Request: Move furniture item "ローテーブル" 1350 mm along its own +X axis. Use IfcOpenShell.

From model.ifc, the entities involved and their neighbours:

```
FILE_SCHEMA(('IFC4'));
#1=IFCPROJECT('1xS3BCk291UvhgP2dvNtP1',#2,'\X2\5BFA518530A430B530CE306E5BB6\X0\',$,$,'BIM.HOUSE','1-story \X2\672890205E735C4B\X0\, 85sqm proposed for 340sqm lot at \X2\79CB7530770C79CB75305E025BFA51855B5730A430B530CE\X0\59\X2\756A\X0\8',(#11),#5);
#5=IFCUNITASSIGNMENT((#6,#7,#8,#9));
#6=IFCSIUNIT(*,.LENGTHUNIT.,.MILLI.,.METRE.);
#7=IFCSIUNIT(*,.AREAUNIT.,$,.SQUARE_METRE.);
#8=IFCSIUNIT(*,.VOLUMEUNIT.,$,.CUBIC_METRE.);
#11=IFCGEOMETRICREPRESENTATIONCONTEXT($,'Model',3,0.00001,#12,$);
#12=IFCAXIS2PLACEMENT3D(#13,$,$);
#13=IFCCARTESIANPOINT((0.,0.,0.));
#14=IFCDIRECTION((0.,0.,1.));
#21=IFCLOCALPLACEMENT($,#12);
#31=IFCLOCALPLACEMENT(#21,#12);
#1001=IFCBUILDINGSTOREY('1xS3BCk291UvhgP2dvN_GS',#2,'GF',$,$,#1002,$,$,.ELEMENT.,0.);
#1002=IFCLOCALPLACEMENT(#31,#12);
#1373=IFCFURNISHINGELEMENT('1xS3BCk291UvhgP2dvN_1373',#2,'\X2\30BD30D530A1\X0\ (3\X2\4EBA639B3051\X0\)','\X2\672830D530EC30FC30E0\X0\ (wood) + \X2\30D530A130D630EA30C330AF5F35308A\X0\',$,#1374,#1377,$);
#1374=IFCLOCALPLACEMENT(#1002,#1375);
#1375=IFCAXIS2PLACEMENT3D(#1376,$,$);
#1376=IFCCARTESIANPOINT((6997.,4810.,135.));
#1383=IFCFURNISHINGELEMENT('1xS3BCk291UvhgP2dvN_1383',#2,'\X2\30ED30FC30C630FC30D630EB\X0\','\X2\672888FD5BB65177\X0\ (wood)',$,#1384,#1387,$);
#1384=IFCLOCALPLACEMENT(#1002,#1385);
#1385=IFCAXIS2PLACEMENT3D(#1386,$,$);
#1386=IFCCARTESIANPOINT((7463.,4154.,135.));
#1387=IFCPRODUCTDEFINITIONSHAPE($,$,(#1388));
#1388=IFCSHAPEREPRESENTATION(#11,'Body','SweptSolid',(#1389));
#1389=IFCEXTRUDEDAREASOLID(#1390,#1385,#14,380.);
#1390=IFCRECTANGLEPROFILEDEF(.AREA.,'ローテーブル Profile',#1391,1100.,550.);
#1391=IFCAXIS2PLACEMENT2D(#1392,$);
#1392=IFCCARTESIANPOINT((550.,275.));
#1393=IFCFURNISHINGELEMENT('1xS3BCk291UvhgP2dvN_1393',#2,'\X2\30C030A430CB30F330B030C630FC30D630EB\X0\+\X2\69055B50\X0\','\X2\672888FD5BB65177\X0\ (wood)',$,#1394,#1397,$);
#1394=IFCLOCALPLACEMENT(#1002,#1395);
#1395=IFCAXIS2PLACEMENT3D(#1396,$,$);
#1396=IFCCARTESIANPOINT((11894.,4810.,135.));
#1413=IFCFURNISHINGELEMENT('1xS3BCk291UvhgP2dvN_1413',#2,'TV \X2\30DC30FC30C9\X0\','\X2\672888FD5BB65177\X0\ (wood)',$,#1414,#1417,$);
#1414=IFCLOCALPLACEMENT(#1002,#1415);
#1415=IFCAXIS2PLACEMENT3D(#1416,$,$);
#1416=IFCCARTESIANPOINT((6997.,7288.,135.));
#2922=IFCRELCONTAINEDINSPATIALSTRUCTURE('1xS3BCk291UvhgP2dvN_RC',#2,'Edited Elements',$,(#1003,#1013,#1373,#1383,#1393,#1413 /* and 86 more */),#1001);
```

```python
import ifcopenshell
import ifcopenshell.api.geometry
import ifcopenshell.util.placement
import ifcopenshell.util.unit

model = ifcopenshell.open("model.ifc")
unit_scale = ifcopenshell.util.unit.calculate_unit_scale(model)

item = model.by_guid("1xS3BCk291UvhgP2dvN_1383")
matrix = ifcopenshell.util.placement.get_local_placement(item.ObjectPlacement)
matrix[:3, 3] += matrix[:3, 0] * 1.35 / unit_scale
ifcopenshell.api.geometry.edit_object_placement(model, product=item, matrix=matrix, is_si=False)

print(ifcopenshell.util.placement.get_local_placement(item.ObjectPlacement).round(3) + 0.0)

model.write("model_v2.ifc")
```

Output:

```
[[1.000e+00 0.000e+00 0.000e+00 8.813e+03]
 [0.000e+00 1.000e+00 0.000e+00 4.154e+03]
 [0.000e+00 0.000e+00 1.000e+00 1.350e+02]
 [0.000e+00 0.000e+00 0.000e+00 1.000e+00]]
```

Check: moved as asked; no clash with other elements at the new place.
